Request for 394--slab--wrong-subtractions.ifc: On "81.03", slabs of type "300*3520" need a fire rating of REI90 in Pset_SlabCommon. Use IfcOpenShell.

First a look at what the model holds.

```python
import ifcopenshell
import ifcopenshell.util.element

model = ifcopenshell.open("394--slab--wrong-subtractions.ifc")
print(model.schema)
storey = next(s for s in model.by_type("IfcBuildingStorey") if s.Name == "81.03")
slabs = [e for e in ifcopenshell.util.element.get_decomposition(storey) if e.is_a("IfcSlab")]
seen = {}
for e in slabs:
    element_type = ifcopenshell.util.element.get_type(e)
    key = (element_type.Name if element_type != e and element_type else None, ifcopenshell.util.element.get_pset(e, "Pset_SlabCommon", "FireRating"))
    seen[key] = seen.get(key, 0) + 1
for (name, value), count in sorted(seen.items(), key=str):
    print(count, "x", name, "|", value)
```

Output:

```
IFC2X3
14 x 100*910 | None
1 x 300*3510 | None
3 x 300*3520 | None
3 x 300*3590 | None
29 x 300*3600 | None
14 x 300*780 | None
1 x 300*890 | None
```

```python
import ifcopenshell
import ifcopenshell.api.pset
import ifcopenshell.util.element

model = ifcopenshell.open("394--slab--wrong-subtractions.ifc")

storey = next(s for s in model.by_type("IfcBuildingStorey") if s.Name == "81.03")
slabs = [e for e in ifcopenshell.util.element.get_decomposition(storey) if e.is_a("IfcSlab")]

count = 0
for e in slabs:
    element_type = ifcopenshell.util.element.get_type(e)
    if element_type in (None, e) or element_type.Name != "300*3520":
        continue
    found = ifcopenshell.util.element.get_pset(e, "Pset_SlabCommon", should_inherit=False)
    if found:
        pset = model.by_id(found["id"])
        if len(ifcopenshell.util.element.get_elements_by_pset(pset)) > 1:
            pset = ifcopenshell.api.pset.unshare_pset(model, products=[e], pset=pset)[0]
    else:
        pset = ifcopenshell.api.pset.add_pset(model, product=e, name="Pset_SlabCommon")
    ifcopenshell.api.pset.edit_pset(model, pset=pset, properties={"FireRating": "REI90"})
    count += 1

print(count, "slabs updated")

model.write("394--slab--wrong-subtractions_rev.ifc")
```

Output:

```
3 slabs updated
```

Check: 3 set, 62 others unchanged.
